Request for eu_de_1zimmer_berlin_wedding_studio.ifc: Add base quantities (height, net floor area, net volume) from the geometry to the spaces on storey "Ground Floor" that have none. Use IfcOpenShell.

First a look at what the model holds.

```python
import ifcopenshell
import ifcopenshell.util.element
import ifcopenshell.util.unit

model = ifcopenshell.open("eu_de_1zimmer_berlin_wedding_studio.ifc")
print(model.schema)
for unit_type in ("LENGTHUNIT", "AREAUNIT", "VOLUMEUNIT"):
    print(unit_type, ifcopenshell.util.unit.calculate_unit_scale(model, unit_type))
storey = next(s for s in model.by_type("IfcBuildingStorey") if s.Name == "Ground Floor")
spaces = [e for e in ifcopenshell.util.element.get_decomposition(storey) if e.is_a("IfcSpace")]
for e in sorted(spaces, key=lambda e: e.id()):
    print(e.id(), e.is_a(), e.Name, list(ifcopenshell.util.element.get_psets(e, qtos_only=True)), sep=" | ")
```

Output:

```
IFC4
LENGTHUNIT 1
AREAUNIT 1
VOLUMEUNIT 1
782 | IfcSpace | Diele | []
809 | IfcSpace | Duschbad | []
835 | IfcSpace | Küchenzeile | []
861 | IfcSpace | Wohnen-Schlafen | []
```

```python
import ifcopenshell
import ifcopenshell.api.pset
import ifcopenshell.geom
import ifcopenshell.util.element
import ifcopenshell.util.shape
import ifcopenshell.util.unit

model = ifcopenshell.open("eu_de_1zimmer_berlin_wedding_studio.ifc")
unit_scale = ifcopenshell.util.unit.calculate_unit_scale(model)
area_scale = ifcopenshell.util.unit.calculate_unit_scale(model, "AREAUNIT")
volume_scale = ifcopenshell.util.unit.calculate_unit_scale(model, "VOLUMEUNIT")
settings = ifcopenshell.geom.settings()

storey = next(s for s in model.by_type("IfcBuildingStorey") if s.Name == "Ground Floor")
spaces = [e for e in ifcopenshell.util.element.get_decomposition(storey) if e.is_a("IfcSpace")]

for e in sorted(spaces, key=lambda e: e.id()):
    if ifcopenshell.util.element.get_psets(e, qtos_only=True, should_inherit=False):
        continue
    # Geometry comes back in metres, in the element's own axes.
    shape = ifcopenshell.geom.create_shape(settings, e)
    values = {
        "Height": ifcopenshell.util.shape.get_z(shape.geometry) / unit_scale,
        "NetFloorArea": ifcopenshell.util.shape.get_footprint_area(shape.geometry) / area_scale,
        "NetVolume": ifcopenshell.util.shape.get_volume(shape.geometry) / volume_scale,
    }
    qto = ifcopenshell.api.pset.add_qto(model, product=e, name="Qto_SpaceBaseQuantities")
    ifcopenshell.api.pset.edit_qto(model, qto=qto, properties=values)
    print(e.id(), {k: round(v, 3) for k, v in values.items()})

model.write("eu_de_1zimmer_berlin_wedding_studio-out.ifc")
```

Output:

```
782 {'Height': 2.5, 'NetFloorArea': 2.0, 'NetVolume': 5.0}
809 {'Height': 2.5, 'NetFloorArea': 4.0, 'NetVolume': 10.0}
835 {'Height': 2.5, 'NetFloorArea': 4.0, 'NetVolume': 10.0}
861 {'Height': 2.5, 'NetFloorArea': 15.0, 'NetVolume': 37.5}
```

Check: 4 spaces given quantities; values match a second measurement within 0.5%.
